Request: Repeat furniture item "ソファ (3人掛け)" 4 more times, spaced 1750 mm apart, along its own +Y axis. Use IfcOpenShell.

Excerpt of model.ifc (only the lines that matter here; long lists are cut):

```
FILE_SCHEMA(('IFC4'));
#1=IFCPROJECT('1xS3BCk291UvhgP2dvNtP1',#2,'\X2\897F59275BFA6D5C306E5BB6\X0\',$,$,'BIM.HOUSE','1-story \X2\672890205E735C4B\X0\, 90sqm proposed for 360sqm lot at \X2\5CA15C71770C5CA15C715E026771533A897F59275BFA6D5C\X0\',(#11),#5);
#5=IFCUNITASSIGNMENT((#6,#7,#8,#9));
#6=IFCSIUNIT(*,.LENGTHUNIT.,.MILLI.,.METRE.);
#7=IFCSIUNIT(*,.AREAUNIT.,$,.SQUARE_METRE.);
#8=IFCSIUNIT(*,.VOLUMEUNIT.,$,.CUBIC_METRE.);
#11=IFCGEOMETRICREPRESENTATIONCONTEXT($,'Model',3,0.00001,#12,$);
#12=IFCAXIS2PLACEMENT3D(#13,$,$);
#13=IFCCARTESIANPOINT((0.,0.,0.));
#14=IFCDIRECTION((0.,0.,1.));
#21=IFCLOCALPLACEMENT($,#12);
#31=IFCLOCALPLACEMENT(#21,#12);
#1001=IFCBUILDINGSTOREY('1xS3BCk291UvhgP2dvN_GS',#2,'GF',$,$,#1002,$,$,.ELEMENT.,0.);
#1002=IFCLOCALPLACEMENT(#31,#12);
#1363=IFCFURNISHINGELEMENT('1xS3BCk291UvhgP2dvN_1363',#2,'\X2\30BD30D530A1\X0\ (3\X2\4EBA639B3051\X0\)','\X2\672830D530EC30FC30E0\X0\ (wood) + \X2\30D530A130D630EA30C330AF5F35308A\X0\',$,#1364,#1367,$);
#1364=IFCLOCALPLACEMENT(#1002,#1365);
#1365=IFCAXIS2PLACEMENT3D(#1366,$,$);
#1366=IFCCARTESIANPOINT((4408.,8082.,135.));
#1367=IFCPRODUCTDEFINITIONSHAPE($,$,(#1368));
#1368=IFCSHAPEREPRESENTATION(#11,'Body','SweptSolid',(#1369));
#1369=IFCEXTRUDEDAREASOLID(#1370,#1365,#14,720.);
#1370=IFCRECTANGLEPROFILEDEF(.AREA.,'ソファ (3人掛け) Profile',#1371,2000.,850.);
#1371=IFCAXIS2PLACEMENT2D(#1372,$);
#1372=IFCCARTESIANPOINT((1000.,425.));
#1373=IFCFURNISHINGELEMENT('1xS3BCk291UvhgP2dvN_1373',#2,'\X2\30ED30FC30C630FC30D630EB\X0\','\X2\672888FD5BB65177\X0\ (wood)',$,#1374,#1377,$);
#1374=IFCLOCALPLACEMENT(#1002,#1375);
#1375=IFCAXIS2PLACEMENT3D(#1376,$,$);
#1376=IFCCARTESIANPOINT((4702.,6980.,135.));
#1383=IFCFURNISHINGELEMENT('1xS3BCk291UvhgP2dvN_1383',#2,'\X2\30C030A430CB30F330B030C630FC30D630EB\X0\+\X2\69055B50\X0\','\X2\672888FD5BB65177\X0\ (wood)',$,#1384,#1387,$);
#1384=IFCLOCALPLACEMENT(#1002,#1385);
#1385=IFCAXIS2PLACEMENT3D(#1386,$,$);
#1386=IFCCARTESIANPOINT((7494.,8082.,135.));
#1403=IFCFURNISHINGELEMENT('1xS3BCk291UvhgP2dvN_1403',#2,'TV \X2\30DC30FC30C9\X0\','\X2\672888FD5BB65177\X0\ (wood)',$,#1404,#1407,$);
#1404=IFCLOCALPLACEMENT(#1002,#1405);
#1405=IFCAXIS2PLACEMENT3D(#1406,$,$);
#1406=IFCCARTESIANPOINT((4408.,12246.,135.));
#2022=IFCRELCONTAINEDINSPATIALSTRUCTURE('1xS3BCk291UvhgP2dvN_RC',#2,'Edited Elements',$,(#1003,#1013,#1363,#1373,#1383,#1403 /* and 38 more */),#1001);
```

```python
import ifcopenshell
import ifcopenshell.api.geometry
import ifcopenshell.api.root
import ifcopenshell.util.element
import ifcopenshell.util.placement
import ifcopenshell.util.unit

model = ifcopenshell.open("model.ifc")
unit_scale = ifcopenshell.util.unit.calculate_unit_scale(model)


def reuse_history(source, copy):
    """copy_class also copies each property set's owner history, people and application; keep the originals."""
    for rel in copy.IsDefinedBy:
        if rel.is_a("IfcRelDefinesByProperties") and (history := rel.RelatingPropertyDefinition.OwnerHistory):
            rel.RelatingPropertyDefinition.OwnerHistory = source.OwnerHistory
            ifcopenshell.util.element.remove_deep2(model, history)


source = model.by_guid("1xS3BCk291UvhgP2dvN_1363")
base = ifcopenshell.util.placement.get_local_placement(source.ObjectPlacement)
step = base[:3, 1] * 1.75 / unit_scale

for i in range(1, 5):
    copy = ifcopenshell.api.root.copy_class(model, product=source)
    copy.Representation = ifcopenshell.util.element.copy_deep(
        model, source.Representation, exclude=["IfcGeometricRepresentationContext", "IfcRepresentationMap"]
    )
    reuse_history(source, copy)
    matrix = base.copy()
    matrix[:3, 3] += i * step
    print("added at", matrix[:3, 3].round(3) + 0.0)
    ifcopenshell.api.geometry.edit_object_placement(model, product=copy, matrix=matrix, is_si=False)

model.write("model_v2.ifc")
```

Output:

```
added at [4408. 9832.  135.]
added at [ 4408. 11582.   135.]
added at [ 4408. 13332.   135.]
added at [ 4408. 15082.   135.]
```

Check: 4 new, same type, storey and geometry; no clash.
